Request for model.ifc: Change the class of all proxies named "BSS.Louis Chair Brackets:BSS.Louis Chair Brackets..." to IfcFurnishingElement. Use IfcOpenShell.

First a look at what the model holds.

```python
import re

import ifcopenshell

model = ifcopenshell.open("model.ifc")
print(model.schema)
seen = {}
for e in model.by_type("IfcBuildingElementProxy"):
    name = re.sub(r":\d+(:\d+)?$", "", e.Name or "")  # drop the element id that some exporters append
    seen[name] = seen.get(name, 0) + 1
for name, count in sorted(seen.items()):
    print(count, "x", name)
```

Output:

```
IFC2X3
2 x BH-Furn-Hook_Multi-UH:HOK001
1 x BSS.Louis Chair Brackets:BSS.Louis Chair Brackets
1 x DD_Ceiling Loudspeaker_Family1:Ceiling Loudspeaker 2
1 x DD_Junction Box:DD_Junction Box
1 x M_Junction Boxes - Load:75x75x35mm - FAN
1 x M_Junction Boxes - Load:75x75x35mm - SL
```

```python
import ifcopenshell
import ifcopenshell.api.root

model = ifcopenshell.open("model.ifc")

proxies = [e.id() for e in model.by_type("IfcBuildingElementProxy") if (e.Name or "").startswith("BSS.Louis Chair Brackets:BSS.Louis Chair Brackets")]
for step_id in proxies:
    proxy = model.by_id(step_id)
    # Reclassifying a typed element also reclassifies its type and the type's other occurrences.
    if proxy.is_a("IfcBuildingElementProxy"):
        ifcopenshell.api.root.reassign_class(model, product=proxy, ifc_class="IfcFurnishingElement")

print(sum(model.by_id(i).is_a("IfcFurnishingElement") for i in proxies), "reclassified")

model.write("model_v2.ifc")
```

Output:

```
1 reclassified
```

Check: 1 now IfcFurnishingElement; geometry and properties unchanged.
